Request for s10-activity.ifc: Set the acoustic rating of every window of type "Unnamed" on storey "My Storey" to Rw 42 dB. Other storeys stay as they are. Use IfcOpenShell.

First a look at what the model holds.

```python
import ifcopenshell
import ifcopenshell.util.element

model = ifcopenshell.open("s10-activity.ifc")
print(model.schema)
storey = next(s for s in model.by_type("IfcBuildingStorey") if s.Name == "My Storey")
windows = [e for e in ifcopenshell.util.element.get_decomposition(storey) if e.is_a("IfcWindow")]
seen = {}
for e in windows:
    element_type = ifcopenshell.util.element.get_type(e)
    key = (element_type.Name if element_type != e and element_type else None, ifcopenshell.util.element.get_pset(e, "Pset_WindowCommon", "AcousticRating"))
    seen[key] = seen.get(key, 0) + 1
for (name, value), count in sorted(seen.items(), key=str):
    print(count, "x", name, "|", value)
```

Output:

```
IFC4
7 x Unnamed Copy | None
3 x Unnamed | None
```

```python
import ifcopenshell
import ifcopenshell.api.pset
import ifcopenshell.util.element

model = ifcopenshell.open("s10-activity.ifc")

storey = next(s for s in model.by_type("IfcBuildingStorey") if s.Name == "My Storey")
windows = [e for e in ifcopenshell.util.element.get_decomposition(storey) if e.is_a("IfcWindow")]

count = 0
for e in windows:
    element_type = ifcopenshell.util.element.get_type(e)
    if element_type in (None, e) or element_type.Name != "Unnamed":
        continue
    # add_pset returns the element's existing set when there is one.
    pset = ifcopenshell.api.pset.add_pset(model, product=e, name="Pset_WindowCommon")
    ifcopenshell.api.pset.edit_pset(model, pset=pset, properties={"AcousticRating": "Rw 42 dB"})
    count += 1

print(count, "windows updated")

model.write("s10-activity_rev.ifc")
```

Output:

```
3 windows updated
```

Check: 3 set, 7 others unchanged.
